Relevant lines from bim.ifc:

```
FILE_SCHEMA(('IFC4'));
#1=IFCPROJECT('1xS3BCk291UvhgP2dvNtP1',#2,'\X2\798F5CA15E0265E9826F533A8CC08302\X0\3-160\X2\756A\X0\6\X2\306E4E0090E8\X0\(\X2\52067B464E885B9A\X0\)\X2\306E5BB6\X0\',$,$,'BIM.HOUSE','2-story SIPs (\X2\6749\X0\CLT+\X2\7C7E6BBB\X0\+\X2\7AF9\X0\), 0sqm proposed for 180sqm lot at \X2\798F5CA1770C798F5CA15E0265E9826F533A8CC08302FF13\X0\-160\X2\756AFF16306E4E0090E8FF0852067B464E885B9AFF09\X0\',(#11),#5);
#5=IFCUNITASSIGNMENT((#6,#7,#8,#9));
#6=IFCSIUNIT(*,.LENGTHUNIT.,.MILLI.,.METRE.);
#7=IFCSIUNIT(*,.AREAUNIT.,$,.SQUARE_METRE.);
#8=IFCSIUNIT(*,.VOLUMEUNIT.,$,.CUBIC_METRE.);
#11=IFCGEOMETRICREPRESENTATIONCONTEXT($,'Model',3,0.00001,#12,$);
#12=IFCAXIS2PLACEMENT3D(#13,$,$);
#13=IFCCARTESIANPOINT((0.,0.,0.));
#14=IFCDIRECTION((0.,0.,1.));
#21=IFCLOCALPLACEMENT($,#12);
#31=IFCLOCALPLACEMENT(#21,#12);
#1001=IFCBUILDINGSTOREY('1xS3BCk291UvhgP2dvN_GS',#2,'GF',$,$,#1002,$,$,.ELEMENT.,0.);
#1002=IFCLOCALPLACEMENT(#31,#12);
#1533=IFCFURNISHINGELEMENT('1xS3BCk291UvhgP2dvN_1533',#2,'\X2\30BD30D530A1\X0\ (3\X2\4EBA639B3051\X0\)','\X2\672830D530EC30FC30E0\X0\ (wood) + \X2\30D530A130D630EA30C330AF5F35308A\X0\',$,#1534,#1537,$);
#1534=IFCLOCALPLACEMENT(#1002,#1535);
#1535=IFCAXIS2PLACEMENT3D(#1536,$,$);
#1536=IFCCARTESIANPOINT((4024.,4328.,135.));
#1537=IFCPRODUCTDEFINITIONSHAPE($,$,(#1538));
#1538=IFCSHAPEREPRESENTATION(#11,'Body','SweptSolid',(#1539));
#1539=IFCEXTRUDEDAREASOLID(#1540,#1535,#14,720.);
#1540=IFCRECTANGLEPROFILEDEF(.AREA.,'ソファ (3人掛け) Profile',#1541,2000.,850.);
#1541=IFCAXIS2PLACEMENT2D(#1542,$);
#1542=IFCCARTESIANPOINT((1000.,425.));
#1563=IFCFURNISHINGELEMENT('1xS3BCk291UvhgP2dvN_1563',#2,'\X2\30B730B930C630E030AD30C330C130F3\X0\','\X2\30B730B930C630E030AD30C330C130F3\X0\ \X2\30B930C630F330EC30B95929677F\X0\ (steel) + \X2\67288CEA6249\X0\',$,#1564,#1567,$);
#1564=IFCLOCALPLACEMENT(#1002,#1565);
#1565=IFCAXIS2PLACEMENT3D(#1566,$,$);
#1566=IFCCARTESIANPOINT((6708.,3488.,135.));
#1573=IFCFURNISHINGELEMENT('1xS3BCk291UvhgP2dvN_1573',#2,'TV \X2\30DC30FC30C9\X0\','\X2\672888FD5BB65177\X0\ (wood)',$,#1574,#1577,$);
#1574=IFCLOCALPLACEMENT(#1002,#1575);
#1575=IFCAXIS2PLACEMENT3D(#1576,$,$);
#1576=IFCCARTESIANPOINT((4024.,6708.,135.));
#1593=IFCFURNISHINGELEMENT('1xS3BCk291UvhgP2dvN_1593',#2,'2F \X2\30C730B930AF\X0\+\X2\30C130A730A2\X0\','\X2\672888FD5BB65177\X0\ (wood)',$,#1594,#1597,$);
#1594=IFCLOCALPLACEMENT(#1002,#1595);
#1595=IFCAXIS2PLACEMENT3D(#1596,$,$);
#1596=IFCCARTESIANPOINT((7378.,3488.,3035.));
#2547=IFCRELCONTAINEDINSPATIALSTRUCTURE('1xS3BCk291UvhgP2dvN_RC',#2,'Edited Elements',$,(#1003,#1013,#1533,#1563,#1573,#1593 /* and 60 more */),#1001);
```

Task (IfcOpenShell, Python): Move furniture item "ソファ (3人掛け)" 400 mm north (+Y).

```python
import ifcopenshell
import ifcopenshell.api.geometry
import ifcopenshell.util.placement
import ifcopenshell.util.unit

model = ifcopenshell.open("bim.ifc")
unit_scale = ifcopenshell.util.unit.calculate_unit_scale(model)

item = model.by_id(1533)
matrix = ifcopenshell.util.placement.get_local_placement(item.ObjectPlacement)
matrix[1, 3] += 0.4 / unit_scale
ifcopenshell.api.geometry.edit_object_placement(model, product=item, matrix=matrix, is_si=False)

print(ifcopenshell.util.placement.get_local_placement(item.ObjectPlacement).round(3) + 0.0)

model.write("bim_edited.ifc")
```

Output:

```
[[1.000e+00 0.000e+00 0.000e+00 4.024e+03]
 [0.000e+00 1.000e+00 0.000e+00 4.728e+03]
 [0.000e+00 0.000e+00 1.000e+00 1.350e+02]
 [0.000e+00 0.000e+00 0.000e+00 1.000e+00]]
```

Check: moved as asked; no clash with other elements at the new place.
